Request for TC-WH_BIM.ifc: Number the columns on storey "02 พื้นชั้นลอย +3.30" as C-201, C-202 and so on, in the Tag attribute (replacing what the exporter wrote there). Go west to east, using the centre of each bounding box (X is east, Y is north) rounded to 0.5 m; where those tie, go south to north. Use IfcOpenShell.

First a look at what the model holds.

```python
import ifcopenshell
import ifcopenshell.util.element
import ifcopenshell.util.placement

model = ifcopenshell.open("TC-WH_BIM.ifc")
print(model.schema)
storey = next(s for s in model.by_type("IfcBuildingStorey") if s.Name == "02 พื้นชั้นลอย +3.30")
columns = [e for e in ifcopenshell.util.element.get_decomposition(storey) if e.is_a("IfcColumn")]
for e in sorted(columns, key=lambda e: e.id()):
    origin = ifcopenshell.util.placement.get_local_placement(e.ObjectPlacement)[:3, 3]
    print(e.id(), e.Tag, e.Name, origin.round(2) + 0.0, sep=" | ")
```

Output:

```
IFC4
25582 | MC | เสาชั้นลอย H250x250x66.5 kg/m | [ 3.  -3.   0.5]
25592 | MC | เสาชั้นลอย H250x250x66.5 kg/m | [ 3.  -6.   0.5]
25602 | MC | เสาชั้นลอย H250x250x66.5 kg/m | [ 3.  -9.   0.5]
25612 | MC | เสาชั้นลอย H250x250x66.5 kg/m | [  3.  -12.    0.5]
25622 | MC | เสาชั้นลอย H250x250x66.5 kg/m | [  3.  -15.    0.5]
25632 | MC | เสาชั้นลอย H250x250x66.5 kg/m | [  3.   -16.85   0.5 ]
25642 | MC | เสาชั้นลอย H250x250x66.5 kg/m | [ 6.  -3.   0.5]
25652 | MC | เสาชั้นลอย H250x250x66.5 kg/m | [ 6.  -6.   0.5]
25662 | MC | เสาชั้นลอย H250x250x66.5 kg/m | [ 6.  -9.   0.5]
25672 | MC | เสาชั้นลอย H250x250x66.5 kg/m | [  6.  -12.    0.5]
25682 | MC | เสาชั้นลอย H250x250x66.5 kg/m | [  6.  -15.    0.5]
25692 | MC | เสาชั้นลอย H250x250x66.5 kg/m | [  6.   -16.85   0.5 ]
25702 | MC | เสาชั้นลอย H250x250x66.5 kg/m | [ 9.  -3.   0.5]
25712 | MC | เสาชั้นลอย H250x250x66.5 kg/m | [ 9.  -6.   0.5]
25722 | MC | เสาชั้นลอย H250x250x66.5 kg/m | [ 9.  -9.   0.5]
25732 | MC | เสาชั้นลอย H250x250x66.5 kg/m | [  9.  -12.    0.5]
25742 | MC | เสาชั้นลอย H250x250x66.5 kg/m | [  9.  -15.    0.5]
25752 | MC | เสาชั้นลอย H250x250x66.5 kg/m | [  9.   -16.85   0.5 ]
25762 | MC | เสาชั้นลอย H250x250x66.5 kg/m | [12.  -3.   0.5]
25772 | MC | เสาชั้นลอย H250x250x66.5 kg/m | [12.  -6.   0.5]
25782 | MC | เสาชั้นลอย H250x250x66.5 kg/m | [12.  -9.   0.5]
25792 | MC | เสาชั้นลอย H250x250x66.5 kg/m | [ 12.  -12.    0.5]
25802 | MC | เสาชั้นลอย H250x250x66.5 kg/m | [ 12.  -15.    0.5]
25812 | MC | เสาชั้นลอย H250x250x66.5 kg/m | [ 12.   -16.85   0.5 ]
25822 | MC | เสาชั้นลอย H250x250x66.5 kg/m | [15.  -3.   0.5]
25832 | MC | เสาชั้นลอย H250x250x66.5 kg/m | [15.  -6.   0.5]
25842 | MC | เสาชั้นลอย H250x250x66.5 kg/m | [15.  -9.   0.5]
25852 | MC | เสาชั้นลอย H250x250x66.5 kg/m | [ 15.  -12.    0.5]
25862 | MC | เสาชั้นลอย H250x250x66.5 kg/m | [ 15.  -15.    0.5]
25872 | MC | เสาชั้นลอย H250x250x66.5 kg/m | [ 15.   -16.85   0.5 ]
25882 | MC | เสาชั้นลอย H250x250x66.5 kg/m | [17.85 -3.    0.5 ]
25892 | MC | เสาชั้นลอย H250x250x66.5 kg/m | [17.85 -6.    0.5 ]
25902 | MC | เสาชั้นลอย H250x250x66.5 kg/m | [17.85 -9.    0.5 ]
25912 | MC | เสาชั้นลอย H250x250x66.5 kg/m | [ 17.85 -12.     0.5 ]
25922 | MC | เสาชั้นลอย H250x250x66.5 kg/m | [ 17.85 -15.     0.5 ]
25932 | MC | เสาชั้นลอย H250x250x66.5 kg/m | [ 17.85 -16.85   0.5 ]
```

```python
import ifcopenshell
import ifcopenshell.geom
import ifcopenshell.util.element
import ifcopenshell.util.shape

model = ifcopenshell.open("TC-WH_BIM.ifc")
settings = ifcopenshell.geom.settings()
settings.set("use-world-coords", True)


def centre(element):
    shape = ifcopenshell.geom.create_shape(settings, element)
    return ifcopenshell.util.shape.get_bbox_centroid(shape.geometry)


storey = next(s for s in model.by_type("IfcBuildingStorey") if s.Name == "02 พื้นชั้นลอย +3.30")
columns = [e for e in ifcopenshell.util.element.get_decomposition(storey) if e.is_a("IfcColumn")]

# Insertion points can sit at a corner or the storey origin, so sort by the geometry (in metres).
centres = {e: centre(e) for e in columns}
columns.sort(key=lambda e: (round(centres[e][0] / 0.5), centres[e][1]))

for i, e in enumerate(columns, start=1):
    number = f"C-2{i:02d}"
    e.Tag = number
    print(e.id(), number)

model.write("TC-WH_BIM-out.ifc")
```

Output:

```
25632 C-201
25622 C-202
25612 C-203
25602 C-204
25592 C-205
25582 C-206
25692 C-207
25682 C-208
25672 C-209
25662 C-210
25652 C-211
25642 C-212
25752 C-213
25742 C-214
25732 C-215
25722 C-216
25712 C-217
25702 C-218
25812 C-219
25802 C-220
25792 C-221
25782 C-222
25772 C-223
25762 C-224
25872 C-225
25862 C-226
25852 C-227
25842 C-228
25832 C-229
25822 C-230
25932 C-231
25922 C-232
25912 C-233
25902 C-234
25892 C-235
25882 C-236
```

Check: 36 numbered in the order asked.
